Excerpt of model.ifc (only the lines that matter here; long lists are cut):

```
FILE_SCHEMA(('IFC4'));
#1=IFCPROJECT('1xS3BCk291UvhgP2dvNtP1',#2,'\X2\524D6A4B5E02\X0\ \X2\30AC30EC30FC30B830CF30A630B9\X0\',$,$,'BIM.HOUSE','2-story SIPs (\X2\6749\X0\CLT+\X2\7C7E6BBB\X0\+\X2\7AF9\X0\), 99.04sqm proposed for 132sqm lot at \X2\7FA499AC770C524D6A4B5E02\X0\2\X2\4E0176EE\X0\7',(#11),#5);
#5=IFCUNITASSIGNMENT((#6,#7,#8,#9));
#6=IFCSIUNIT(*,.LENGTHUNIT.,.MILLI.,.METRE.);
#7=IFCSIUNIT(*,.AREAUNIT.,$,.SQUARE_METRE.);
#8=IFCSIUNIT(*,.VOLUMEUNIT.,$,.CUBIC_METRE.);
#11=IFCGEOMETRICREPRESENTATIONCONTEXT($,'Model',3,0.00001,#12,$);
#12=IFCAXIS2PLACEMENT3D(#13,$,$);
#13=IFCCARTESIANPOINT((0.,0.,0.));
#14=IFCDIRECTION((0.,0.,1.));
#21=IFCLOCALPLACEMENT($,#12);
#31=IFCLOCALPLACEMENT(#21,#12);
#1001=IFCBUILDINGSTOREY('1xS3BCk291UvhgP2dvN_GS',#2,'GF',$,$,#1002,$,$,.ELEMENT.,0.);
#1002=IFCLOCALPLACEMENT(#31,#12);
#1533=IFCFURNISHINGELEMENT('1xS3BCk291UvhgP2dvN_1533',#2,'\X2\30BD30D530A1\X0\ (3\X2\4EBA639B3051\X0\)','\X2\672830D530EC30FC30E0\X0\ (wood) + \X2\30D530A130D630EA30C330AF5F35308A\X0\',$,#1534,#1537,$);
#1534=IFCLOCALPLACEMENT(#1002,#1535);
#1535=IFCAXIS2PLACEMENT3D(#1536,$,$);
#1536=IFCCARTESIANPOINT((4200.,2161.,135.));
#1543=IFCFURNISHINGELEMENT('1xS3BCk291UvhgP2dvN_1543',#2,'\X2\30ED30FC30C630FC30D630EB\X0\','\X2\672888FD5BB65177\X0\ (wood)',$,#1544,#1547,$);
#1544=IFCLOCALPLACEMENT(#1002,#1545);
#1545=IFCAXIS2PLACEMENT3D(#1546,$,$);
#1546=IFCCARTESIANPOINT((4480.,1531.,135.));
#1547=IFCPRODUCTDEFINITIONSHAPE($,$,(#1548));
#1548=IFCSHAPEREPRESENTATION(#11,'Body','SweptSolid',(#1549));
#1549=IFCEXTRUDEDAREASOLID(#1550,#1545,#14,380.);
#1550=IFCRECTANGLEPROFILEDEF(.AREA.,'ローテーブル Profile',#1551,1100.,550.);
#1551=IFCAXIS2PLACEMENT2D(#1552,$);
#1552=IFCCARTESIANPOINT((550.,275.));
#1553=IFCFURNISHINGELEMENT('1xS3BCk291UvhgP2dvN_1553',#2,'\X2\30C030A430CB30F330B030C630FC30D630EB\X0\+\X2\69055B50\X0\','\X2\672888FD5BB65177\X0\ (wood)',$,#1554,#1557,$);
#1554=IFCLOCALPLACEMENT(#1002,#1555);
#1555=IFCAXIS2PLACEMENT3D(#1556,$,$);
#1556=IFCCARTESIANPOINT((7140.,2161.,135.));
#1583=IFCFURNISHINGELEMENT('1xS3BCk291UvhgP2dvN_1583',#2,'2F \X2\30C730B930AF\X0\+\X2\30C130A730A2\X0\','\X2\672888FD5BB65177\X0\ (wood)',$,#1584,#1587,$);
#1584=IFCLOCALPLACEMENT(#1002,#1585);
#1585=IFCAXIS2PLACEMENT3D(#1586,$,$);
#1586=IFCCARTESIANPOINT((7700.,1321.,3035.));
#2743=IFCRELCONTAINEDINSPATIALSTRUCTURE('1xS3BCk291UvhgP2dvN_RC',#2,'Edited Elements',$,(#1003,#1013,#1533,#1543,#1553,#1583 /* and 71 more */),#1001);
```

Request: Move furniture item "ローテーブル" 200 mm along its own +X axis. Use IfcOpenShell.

```python
import ifcopenshell
import ifcopenshell.api.geometry
import ifcopenshell.util.placement
import ifcopenshell.util.unit

model = ifcopenshell.open("model.ifc")
unit_scale = ifcopenshell.util.unit.calculate_unit_scale(model)

item = model.by_guid("1xS3BCk291UvhgP2dvN_1543")
matrix = ifcopenshell.util.placement.get_local_placement(item.ObjectPlacement)
matrix[:3, 3] += matrix[:3, 0] * 0.2 / unit_scale
ifcopenshell.api.geometry.edit_object_placement(model, product=item, matrix=matrix, is_si=False)

print(ifcopenshell.util.placement.get_local_placement(item.ObjectPlacement).round(3) + 0.0)

model.write("model_edited.ifc")
```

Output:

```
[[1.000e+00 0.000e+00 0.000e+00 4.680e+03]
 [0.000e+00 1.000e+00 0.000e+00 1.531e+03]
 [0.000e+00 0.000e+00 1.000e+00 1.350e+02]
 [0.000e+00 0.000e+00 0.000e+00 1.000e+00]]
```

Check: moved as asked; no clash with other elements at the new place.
